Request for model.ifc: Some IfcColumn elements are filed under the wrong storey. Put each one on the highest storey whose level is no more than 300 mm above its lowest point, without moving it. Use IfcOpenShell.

First a look at what the model holds.

```python
import ifcopenshell
import ifcopenshell.util.element
import ifcopenshell.util.placement

model = ifcopenshell.open("model.ifc")
print(model.schema)
for storey in model.by_type("IfcBuildingStorey"):
    level = ifcopenshell.util.placement.get_storey_elevation(storey)
    count = sum(e.is_a("IfcColumn") for e in ifcopenshell.util.element.get_contained(storey))
    print(storey.id(), storey.Name, round(level, 3), count, sep=" | ")
```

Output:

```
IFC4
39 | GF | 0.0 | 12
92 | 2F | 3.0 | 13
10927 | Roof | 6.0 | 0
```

```python
import ifcopenshell
import ifcopenshell.api.spatial
import ifcopenshell.geom
import ifcopenshell.util.element
import ifcopenshell.util.placement
import ifcopenshell.util.shape
import ifcopenshell.util.unit

model = ifcopenshell.open("model.ifc")
unit_scale = ifcopenshell.util.unit.calculate_unit_scale(model)
settings = ifcopenshell.geom.settings()

levels = sorted(
    ((ifcopenshell.util.placement.get_storey_elevation(s) * unit_scale, s) for s in model.by_type("IfcBuildingStorey")),
    key=lambda pair: pair[0],
)

for e in model.by_type("IfcColumn"):
    current = e.ContainedInStructure[0].RelatingStructure if e.ContainedInStructure else None
    if current is None or not current.is_a("IfcBuildingStorey"):
        continue
    shape = ifcopenshell.geom.create_shape(settings, e)
    bottom = ifcopenshell.util.shape.get_shape_bottom_elevation(shape, shape.geometry)
    below = [s for level, s in levels if level <= bottom + 0.3]
    storey = below[-1] if below else levels[0][1]
    if storey != current:
        # assign_container keeps the world position.
        ifcopenshell.api.spatial.assign_container(model, products=[e], relating_structure=storey)
        print(e.id(), current.Name, "->", storey.Name)

model.write("model_rev.ifc")
```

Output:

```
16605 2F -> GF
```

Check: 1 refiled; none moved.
